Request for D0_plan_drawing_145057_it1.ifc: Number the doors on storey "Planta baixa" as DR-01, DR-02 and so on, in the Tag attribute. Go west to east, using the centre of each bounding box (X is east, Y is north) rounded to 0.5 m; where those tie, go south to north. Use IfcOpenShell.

First a look at what the model holds.

```python
import ifcopenshell
import ifcopenshell.util.element
import ifcopenshell.util.placement

model = ifcopenshell.open("D0_plan_drawing_145057_it1.ifc")
print(model.schema)
storey = next(s for s in model.by_type("IfcBuildingStorey") if s.Name == "Planta baixa")
doors = [e for e in ifcopenshell.util.element.get_decomposition(storey) if e.is_a("IfcDoor")]
for e in sorted(doors, key=lambda e: e.id()):
    origin = ifcopenshell.util.placement.get_local_placement(e.ObjectPlacement)[:3, 3]
    print(e.id(), e.Tag, e.Name, origin.round(2) + 0.0, sep=" | ")
```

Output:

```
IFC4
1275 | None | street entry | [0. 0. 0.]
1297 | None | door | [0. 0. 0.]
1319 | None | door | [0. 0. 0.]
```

```python
import ifcopenshell
import ifcopenshell.geom
import ifcopenshell.util.element
import ifcopenshell.util.shape

model = ifcopenshell.open("D0_plan_drawing_145057_it1.ifc")
settings = ifcopenshell.geom.settings()
settings.set("use-world-coords", True)


def centre(element):
    shape = ifcopenshell.geom.create_shape(settings, element)
    return ifcopenshell.util.shape.get_bbox_centroid(shape.geometry)


storey = next(s for s in model.by_type("IfcBuildingStorey") if s.Name == "Planta baixa")
doors = [e for e in ifcopenshell.util.element.get_decomposition(storey) if e.is_a("IfcDoor")]

# Insertion points can sit at a corner or the storey origin, so sort by the geometry (in metres).
centres = {e: centre(e) for e in doors}
doors.sort(key=lambda e: (round(centres[e][0] / 0.5), centres[e][1]))

for i, e in enumerate(doors, start=1):
    number = f"DR-{i:02d}"
    e.Tag = number
    print(e.id(), number)

model.write("D0_plan_drawing_145057_it1-out.ifc")
```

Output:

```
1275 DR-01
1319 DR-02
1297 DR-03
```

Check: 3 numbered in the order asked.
